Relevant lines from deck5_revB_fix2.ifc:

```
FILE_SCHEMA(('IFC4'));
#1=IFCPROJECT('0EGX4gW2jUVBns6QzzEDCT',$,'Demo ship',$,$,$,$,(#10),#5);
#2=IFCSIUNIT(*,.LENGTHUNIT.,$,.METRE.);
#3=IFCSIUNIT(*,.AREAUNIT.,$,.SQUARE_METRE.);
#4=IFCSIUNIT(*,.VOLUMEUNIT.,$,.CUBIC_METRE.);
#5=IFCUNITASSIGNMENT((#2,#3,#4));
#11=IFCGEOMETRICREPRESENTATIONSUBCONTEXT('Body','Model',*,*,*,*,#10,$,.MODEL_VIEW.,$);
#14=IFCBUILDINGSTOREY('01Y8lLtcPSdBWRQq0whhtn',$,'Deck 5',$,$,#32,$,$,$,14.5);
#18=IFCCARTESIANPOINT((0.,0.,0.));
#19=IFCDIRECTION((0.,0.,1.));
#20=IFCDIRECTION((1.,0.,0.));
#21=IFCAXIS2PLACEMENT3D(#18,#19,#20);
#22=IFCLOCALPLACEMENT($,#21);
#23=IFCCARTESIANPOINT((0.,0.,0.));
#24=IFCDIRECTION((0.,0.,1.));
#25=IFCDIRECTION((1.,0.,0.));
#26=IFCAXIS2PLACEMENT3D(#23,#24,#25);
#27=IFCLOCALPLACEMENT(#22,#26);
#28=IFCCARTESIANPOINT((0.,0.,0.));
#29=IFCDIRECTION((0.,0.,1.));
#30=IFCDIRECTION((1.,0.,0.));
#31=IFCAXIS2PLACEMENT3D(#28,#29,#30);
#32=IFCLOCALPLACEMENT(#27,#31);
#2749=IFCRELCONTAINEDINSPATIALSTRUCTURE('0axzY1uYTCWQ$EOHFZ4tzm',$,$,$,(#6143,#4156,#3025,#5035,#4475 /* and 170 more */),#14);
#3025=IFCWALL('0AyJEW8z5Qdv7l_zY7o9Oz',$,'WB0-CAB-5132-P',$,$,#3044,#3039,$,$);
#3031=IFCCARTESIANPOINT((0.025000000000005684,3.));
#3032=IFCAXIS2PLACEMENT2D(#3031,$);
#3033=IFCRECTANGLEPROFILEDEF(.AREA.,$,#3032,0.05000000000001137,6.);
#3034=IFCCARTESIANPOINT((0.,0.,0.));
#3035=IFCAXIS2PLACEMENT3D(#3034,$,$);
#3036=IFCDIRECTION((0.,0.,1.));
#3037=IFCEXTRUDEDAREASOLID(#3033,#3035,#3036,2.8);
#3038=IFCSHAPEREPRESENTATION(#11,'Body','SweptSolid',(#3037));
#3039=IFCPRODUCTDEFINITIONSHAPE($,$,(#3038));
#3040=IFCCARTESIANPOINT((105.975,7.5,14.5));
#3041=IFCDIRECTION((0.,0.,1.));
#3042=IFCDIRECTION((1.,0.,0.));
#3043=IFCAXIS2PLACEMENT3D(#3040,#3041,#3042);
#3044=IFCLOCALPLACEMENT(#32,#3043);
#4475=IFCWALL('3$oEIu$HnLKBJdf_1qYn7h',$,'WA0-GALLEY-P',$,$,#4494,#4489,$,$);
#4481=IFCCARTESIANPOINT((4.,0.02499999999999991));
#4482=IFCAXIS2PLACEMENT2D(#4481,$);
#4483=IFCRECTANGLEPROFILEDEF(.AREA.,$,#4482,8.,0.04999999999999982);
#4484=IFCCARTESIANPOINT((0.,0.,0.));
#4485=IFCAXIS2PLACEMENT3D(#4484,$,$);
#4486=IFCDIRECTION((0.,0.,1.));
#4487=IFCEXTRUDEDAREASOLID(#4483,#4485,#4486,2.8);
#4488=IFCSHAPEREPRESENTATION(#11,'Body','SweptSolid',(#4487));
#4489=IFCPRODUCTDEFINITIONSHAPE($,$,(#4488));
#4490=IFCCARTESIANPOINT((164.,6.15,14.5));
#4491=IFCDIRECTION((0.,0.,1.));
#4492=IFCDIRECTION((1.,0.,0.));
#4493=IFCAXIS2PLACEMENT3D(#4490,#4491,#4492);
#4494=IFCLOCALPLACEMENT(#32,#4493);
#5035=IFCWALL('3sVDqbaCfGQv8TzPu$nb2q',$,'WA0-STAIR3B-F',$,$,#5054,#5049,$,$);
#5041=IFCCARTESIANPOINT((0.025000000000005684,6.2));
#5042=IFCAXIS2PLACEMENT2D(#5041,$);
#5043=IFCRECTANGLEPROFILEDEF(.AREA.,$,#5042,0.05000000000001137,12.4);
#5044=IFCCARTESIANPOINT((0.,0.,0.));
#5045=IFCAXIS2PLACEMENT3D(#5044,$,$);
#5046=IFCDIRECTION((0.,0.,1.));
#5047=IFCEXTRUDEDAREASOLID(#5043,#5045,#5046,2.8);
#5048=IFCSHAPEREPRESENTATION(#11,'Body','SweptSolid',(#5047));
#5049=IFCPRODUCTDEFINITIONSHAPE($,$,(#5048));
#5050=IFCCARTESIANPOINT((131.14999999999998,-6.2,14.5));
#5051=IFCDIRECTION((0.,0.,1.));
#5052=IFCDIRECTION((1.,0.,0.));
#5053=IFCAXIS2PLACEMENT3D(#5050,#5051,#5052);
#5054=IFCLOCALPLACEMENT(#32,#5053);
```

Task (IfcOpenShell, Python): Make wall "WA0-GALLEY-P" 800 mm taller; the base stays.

```python
import ifcopenshell
import ifcopenshell.geom
import ifcopenshell.util.representation
import ifcopenshell.util.shape
import ifcopenshell.util.unit

model = ifcopenshell.open("deck5_revB_fix2.ifc")
unit_scale = ifcopenshell.util.unit.calculate_unit_scale(model)
settings = ifcopenshell.geom.settings()


def volume(element):
    """Net volume in cubic metres, openings subtracted."""
    shape = ifcopenshell.geom.create_shape(settings, element)
    return ifcopenshell.util.shape.get_volume(shape.geometry)


wall = model.by_guid("3$oEIu$HnLKBJdf_1qYn7h")
before = volume(wall)

body = ifcopenshell.util.representation.get_representation(wall, "Model", "Body")
solid = body.Items[0]
old_height = solid.Depth
solid.Depth += 0.8 / unit_scale
after = volume(wall)

print(f"height {old_height:g} -> {solid.Depth:g}, volume {before:.3f} -> {after:.3f} m3")

model.write("deck5_revB_fix2-out.ifc")
```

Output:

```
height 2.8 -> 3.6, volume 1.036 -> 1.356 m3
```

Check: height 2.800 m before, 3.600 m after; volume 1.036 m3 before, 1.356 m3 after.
